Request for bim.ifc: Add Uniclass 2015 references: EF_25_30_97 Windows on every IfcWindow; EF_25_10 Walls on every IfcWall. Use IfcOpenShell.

First a look at what the model holds.

```python
import ifcopenshell

model = ifcopenshell.open("bim.ifc")
print(model.schema)
print("classifications:", [c.Name for c in model.by_type("IfcClassification")])
for ifc_class in ("IfcDoor", "IfcRoof", "IfcStair", "IfcWall", "IfcWindow"):
    print(ifc_class, len(model.by_type(ifc_class)))
```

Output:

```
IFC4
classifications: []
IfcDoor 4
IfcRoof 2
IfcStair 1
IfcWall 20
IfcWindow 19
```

```python
import ifcopenshell
import ifcopenshell.api.classification

model = ifcopenshell.open("bim.ifc")

system = ifcopenshell.api.classification.add_classification(model, classification="Uniclass 2015")

codes = {
    "IfcWindow": ("EF_25_30_97", "Windows"),
    "IfcWall": ("EF_25_10", "Walls"),
}
for ifc_class, (code, name) in codes.items():
    products = model.by_type(ifc_class)
    ifcopenshell.api.classification.add_reference(
        model, products=products, classification=system, identification=code, name=name
    )
    print(code, len(products))

model.write("bim-out.ifc")
```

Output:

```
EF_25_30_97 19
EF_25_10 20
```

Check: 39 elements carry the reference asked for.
